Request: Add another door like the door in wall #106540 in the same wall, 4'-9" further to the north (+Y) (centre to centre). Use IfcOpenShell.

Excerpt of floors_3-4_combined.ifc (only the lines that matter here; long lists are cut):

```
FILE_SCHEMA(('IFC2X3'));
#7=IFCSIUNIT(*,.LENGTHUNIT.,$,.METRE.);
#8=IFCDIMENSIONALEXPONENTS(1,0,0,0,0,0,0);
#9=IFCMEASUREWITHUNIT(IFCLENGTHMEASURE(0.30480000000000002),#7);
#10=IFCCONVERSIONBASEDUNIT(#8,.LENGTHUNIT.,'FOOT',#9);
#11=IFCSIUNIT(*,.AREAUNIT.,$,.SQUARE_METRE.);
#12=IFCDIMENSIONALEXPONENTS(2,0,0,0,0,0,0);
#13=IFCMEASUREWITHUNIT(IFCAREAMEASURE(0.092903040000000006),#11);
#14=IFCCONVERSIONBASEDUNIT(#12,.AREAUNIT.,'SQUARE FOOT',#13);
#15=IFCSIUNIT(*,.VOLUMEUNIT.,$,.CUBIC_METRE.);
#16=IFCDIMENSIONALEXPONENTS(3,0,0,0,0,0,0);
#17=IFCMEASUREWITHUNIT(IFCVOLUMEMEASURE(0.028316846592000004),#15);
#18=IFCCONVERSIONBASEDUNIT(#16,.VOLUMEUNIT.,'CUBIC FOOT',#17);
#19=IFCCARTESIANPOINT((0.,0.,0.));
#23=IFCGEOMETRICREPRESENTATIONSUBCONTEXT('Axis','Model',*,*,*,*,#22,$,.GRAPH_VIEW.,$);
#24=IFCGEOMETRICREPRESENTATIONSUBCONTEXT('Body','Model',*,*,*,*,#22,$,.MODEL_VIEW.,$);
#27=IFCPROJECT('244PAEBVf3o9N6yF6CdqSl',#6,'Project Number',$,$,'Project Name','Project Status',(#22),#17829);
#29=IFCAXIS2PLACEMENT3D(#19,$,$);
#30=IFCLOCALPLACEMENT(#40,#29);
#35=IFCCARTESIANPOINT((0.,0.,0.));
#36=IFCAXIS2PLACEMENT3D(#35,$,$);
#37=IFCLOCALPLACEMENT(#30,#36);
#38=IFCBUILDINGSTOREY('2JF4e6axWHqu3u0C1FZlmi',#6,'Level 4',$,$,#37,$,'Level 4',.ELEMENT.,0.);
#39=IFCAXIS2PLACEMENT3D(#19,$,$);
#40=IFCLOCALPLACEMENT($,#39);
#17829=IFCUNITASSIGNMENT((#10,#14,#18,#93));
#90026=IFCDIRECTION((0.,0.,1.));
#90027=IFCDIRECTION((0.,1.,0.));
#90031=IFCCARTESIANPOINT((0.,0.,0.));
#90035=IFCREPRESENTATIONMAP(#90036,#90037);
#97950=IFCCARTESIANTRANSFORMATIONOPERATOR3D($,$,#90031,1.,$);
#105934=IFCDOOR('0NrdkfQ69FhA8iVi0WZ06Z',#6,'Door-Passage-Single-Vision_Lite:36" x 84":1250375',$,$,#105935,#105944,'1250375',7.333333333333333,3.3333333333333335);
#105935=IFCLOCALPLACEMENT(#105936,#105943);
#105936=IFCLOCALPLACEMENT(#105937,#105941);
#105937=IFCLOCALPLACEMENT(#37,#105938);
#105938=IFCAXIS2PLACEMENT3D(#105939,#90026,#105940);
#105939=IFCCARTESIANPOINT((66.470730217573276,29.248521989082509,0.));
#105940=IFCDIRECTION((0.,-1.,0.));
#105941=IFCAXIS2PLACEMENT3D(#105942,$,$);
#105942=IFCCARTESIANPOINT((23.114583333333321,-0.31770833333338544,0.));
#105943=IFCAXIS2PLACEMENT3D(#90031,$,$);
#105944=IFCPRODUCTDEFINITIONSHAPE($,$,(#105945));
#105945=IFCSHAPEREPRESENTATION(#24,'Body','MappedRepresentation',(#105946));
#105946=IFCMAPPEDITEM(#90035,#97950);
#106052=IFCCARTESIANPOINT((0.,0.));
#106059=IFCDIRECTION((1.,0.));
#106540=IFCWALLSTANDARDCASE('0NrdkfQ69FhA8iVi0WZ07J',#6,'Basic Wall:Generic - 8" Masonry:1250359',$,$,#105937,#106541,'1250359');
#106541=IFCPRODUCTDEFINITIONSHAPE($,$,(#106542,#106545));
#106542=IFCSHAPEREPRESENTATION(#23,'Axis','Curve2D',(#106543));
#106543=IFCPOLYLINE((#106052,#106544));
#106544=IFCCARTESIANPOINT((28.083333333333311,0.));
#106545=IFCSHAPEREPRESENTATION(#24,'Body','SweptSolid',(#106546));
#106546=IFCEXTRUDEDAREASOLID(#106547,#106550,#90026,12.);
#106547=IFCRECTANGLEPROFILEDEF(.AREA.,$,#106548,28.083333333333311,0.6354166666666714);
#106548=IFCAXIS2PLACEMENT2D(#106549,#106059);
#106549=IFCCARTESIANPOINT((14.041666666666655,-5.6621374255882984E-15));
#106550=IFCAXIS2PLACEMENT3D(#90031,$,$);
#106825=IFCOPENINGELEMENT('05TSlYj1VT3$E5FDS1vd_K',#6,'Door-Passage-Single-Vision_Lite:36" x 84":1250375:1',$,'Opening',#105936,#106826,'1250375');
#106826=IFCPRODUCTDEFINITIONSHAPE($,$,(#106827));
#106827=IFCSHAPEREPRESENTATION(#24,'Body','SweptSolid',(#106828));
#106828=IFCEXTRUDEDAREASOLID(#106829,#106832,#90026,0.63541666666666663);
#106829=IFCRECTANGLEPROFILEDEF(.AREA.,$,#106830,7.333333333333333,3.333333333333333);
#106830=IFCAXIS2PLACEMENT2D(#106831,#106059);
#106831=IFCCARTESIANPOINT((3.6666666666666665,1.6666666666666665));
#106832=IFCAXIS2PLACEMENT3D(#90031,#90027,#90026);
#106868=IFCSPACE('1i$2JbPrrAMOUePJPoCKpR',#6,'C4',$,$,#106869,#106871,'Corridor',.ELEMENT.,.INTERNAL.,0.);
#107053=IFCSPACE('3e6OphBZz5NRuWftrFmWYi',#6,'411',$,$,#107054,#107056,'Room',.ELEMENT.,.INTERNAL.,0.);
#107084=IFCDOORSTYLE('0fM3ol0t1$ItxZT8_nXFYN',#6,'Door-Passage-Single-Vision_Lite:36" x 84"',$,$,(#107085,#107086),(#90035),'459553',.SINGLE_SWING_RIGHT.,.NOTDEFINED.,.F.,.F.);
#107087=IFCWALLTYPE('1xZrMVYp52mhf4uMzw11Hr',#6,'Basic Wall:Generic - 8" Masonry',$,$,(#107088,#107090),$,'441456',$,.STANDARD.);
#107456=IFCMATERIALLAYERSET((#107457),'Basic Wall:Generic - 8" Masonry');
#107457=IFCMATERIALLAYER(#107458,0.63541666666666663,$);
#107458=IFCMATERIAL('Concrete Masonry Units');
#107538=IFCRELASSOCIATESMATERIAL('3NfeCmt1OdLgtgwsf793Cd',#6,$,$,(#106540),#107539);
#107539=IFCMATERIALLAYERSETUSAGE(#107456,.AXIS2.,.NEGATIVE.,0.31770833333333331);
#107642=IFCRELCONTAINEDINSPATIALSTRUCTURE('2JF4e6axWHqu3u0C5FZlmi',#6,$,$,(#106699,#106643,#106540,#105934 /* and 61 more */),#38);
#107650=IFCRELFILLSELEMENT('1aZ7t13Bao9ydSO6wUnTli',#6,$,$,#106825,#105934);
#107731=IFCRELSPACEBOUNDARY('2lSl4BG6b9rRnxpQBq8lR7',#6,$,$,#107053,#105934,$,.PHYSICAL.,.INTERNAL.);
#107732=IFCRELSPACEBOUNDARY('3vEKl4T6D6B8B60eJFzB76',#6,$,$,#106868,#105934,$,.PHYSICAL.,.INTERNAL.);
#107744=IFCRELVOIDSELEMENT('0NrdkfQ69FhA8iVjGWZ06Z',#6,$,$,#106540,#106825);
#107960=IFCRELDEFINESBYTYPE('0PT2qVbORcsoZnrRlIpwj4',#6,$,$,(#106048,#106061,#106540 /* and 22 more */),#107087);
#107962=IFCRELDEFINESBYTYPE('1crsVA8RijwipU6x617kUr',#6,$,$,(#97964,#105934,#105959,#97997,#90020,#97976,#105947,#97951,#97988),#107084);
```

```python
import ifcopenshell
import ifcopenshell.api.feature
import ifcopenshell.api.geometry
import ifcopenshell.api.root
import ifcopenshell.geom
import ifcopenshell.util.element
import ifcopenshell.util.placement
import ifcopenshell.util.shape
import ifcopenshell.util.unit

model = ifcopenshell.open("floors_3-4_combined.ifc")
unit_scale = ifcopenshell.util.unit.calculate_unit_scale(model)
settings = ifcopenshell.geom.settings()


def volume(element):
    """Net volume in cubic metres, openings subtracted."""
    shape = ifcopenshell.geom.create_shape(settings, element)
    return ifcopenshell.util.shape.get_volume(shape.geometry)


def reuse_history(source, copy):
    """copy_class also copies each property set's owner history, people and application; keep the originals."""
    for rel in copy.IsDefinedBy:
        if rel.is_a("IfcRelDefinesByProperties") and (history := rel.RelatingPropertyDefinition.OwnerHistory):
            rel.RelatingPropertyDefinition.OwnerHistory = source.OwnerHistory
            ifcopenshell.util.element.remove_deep2(model, history)


door = model.by_guid("0NrdkfQ69FhA8iVi0WZ06Z")
opening = door.FillsVoids[0].RelatingOpeningElement
wall = opening.VoidsElements[0].RelatingBuildingElement
before = volume(wall)
shift = ifcopenshell.util.placement.get_local_placement(wall.ObjectPlacement)[:3, 0] * -57 * 0.0254 / unit_scale

# copy_class copies the void relationship, type, container and properties, but no geometry.
new_opening = ifcopenshell.api.root.copy_class(model, product=opening)
new_opening.Representation = ifcopenshell.util.element.copy_deep(
    model, opening.Representation, exclude=["IfcGeometricRepresentationContext", "IfcRepresentationMap"]
)
new_opening.Name = 'Door-Passage-Single-Vision_Lite:36" x 84"'
new_opening.Tag = None
new_door = ifcopenshell.api.root.copy_class(model, product=door)
new_door.Representation = ifcopenshell.util.element.copy_deep(
    model, door.Representation, exclude=["IfcGeometricRepresentationContext", "IfcRepresentationMap"]
)
new_door.Name = 'Door-Passage-Single-Vision_Lite:36" x 84"'
new_door.Tag = None
reuse_history(door, new_door)
fills = ifcopenshell.api.feature.add_filling(model, opening=new_opening, element=new_door)
fills.OwnerHistory = new_door.OwnerHistory  # required in IFC2X3

for old, new in ((opening, new_opening), (door, new_door)):
    matrix = ifcopenshell.util.placement.get_local_placement(old.ObjectPlacement)
    matrix[:3, 3] += shift
    ifcopenshell.api.geometry.edit_object_placement(model, product=new, matrix=matrix, is_si=False)

after = volume(wall)

print(f"wall volume {before:.3f} -> {after:.3f} m3")

model.write("floors_3-4_combined-out.ifc")
```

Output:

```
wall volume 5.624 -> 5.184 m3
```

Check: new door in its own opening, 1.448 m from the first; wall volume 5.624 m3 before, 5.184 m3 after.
